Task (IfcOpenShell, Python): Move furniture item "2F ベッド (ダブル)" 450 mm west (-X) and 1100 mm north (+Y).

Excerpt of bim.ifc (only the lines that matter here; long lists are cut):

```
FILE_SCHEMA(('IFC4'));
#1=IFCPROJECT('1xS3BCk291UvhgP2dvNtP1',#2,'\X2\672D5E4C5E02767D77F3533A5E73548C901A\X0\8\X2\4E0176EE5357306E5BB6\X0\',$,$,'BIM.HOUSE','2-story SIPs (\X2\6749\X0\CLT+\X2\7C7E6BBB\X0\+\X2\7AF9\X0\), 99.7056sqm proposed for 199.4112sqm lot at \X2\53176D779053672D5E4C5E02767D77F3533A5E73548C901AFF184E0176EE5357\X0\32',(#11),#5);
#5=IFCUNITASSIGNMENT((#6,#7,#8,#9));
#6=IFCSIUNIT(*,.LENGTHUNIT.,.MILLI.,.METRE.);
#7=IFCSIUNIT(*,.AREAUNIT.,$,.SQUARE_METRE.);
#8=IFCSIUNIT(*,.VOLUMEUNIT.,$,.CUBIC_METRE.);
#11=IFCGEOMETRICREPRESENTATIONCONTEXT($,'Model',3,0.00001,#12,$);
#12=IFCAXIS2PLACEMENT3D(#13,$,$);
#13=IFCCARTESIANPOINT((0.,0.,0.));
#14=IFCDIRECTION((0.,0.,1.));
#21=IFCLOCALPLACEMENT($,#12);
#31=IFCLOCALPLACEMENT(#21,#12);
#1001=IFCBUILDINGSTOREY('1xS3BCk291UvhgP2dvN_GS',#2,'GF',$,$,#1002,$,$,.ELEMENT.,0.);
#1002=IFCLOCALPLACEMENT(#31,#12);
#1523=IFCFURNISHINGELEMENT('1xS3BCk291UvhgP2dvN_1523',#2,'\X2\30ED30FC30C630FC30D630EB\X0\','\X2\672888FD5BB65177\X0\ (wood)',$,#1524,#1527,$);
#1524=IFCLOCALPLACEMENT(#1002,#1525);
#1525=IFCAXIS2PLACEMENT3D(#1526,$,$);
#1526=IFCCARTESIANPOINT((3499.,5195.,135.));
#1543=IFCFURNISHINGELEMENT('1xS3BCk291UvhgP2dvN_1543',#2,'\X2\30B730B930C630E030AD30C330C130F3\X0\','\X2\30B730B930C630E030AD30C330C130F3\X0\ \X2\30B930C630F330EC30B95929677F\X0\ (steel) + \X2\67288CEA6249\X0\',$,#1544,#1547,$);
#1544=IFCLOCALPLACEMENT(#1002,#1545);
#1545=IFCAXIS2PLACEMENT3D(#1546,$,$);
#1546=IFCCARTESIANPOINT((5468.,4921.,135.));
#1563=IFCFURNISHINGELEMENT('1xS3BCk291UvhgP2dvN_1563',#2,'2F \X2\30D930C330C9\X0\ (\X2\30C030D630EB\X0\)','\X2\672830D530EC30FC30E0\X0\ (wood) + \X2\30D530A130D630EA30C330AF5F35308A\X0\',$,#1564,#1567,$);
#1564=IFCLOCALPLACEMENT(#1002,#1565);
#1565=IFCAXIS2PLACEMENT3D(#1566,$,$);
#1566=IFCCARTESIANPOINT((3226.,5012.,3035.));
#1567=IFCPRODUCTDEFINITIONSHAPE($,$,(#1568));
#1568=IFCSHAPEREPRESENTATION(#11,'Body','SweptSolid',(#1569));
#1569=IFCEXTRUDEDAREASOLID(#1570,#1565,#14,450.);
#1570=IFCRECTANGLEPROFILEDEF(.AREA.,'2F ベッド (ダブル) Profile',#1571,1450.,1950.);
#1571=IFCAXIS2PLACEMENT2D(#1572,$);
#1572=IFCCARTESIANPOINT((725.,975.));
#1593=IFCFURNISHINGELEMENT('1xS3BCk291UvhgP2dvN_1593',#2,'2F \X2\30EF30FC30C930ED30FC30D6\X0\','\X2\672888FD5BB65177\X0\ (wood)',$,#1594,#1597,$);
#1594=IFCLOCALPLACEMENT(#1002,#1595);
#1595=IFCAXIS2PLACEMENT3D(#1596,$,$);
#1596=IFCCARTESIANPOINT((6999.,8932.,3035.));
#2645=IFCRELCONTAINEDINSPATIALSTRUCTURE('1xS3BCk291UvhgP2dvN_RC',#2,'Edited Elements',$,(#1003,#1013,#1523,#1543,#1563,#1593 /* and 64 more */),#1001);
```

```python
import ifcopenshell
import ifcopenshell.api.geometry
import ifcopenshell.util.placement
import ifcopenshell.util.unit

model = ifcopenshell.open("bim.ifc")
unit_scale = ifcopenshell.util.unit.calculate_unit_scale(model)

item = model.by_id(1563)
matrix = ifcopenshell.util.placement.get_local_placement(item.ObjectPlacement)
matrix[0, 3] -= 0.45 / unit_scale
matrix[1, 3] += 1.1 / unit_scale
ifcopenshell.api.geometry.edit_object_placement(model, product=item, matrix=matrix, is_si=False)

print(ifcopenshell.util.placement.get_local_placement(item.ObjectPlacement).round(3) + 0.0)

model.write("bim_edited.ifc")
```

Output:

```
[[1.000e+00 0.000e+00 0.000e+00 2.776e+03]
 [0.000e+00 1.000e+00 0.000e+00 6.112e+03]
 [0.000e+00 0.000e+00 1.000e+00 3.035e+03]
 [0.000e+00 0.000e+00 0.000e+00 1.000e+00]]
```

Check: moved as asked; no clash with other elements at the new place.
